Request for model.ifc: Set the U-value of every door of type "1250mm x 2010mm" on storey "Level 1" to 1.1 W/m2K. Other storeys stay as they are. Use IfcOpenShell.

First a look at what the model holds.

```python
import ifcopenshell
import ifcopenshell.util.element

model = ifcopenshell.open("model.ifc")
print(model.schema)
storey = next(s for s in model.by_type("IfcBuildingStorey") if s.Name == "Level 1")
doors = [e for e in ifcopenshell.util.element.get_decomposition(storey) if e.is_a("IfcDoor")]
seen = {}
for e in doors:
    element_type = ifcopenshell.util.element.get_type(e)
    key = (element_type.Name if element_type != e and element_type else None, ifcopenshell.util.element.get_pset(e, "Pset_DoorCommon", "ThermalTransmittance"))
    seen[key] = seen.get(key, 0) + 1
for (name, value), count in sorted(seen.items(), key=str):
    print(count, "x", name, "|", value)
```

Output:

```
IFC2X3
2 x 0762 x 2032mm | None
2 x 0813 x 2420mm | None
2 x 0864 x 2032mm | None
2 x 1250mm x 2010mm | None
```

```python
import ifcopenshell
import ifcopenshell.api.pset
import ifcopenshell.util.element

model = ifcopenshell.open("model.ifc")

storey = next(s for s in model.by_type("IfcBuildingStorey") if s.Name == "Level 1")
doors = [e for e in ifcopenshell.util.element.get_decomposition(storey) if e.is_a("IfcDoor")]

count = 0
for e in doors:
    element_type = ifcopenshell.util.element.get_type(e)
    if element_type in (None, e) or element_type.Name != "1250mm x 2010mm":
        continue
    # add_pset returns the element's existing set when there is one.
    pset = ifcopenshell.api.pset.add_pset(model, product=e, name="Pset_DoorCommon")
    ifcopenshell.api.pset.edit_pset(model, pset=pset, properties={"ThermalTransmittance": 1.1})
    count += 1

print(count, "doors updated")

model.write("model_rev.ifc")
```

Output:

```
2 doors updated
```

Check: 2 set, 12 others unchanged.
